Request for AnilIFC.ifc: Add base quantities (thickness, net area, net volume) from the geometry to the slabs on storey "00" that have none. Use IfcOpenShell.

First a look at what the model holds.

```python
import ifcopenshell
import ifcopenshell.util.element
import ifcopenshell.util.unit

model = ifcopenshell.open("AnilIFC.ifc")
print(model.schema)
for unit_type in ("LENGTHUNIT", "AREAUNIT", "VOLUMEUNIT"):
    print(unit_type, ifcopenshell.util.unit.calculate_unit_scale(model, unit_type))
storey = next(s for s in model.by_type("IfcBuildingStorey") if s.Name == "00")
slabs = [e for e in ifcopenshell.util.element.get_decomposition(storey) if e.is_a("IfcSlab")]
for e in sorted(slabs, key=lambda e: e.id()):
    print(e.id(), e.is_a(), e.Name, list(ifcopenshell.util.element.get_psets(e, qtos_only=True)), sep=" | ")
```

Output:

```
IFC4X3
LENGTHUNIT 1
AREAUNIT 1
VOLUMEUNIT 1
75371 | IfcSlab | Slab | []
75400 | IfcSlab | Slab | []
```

```python
import ifcopenshell
import ifcopenshell.api.pset
import ifcopenshell.geom
import ifcopenshell.util.element
import ifcopenshell.util.shape
import ifcopenshell.util.unit

model = ifcopenshell.open("AnilIFC.ifc")
unit_scale = ifcopenshell.util.unit.calculate_unit_scale(model)
area_scale = ifcopenshell.util.unit.calculate_unit_scale(model, "AREAUNIT")
volume_scale = ifcopenshell.util.unit.calculate_unit_scale(model, "VOLUMEUNIT")
settings = ifcopenshell.geom.settings()

storey = next(s for s in model.by_type("IfcBuildingStorey") if s.Name == "00")
slabs = [e for e in ifcopenshell.util.element.get_decomposition(storey) if e.is_a("IfcSlab")]

for e in sorted(slabs, key=lambda e: e.id()):
    if ifcopenshell.util.element.get_psets(e, qtos_only=True, should_inherit=False):
        continue
    # Geometry comes back in metres, in the element's own axes.
    shape = ifcopenshell.geom.create_shape(settings, e)
    values = {
        "Width": ifcopenshell.util.shape.get_z(shape.geometry) / unit_scale,
        "NetArea": ifcopenshell.util.shape.get_footprint_area(shape.geometry) / area_scale,
        "NetVolume": ifcopenshell.util.shape.get_volume(shape.geometry) / volume_scale,
    }
    qto = ifcopenshell.api.pset.add_qto(model, product=e, name="Qto_SlabBaseQuantities")
    ifcopenshell.api.pset.edit_qto(model, qto=qto, properties=values)
    print(e.id(), {k: round(v, 3) for k, v in values.items()})

model.write("AnilIFC_v2.ifc")
```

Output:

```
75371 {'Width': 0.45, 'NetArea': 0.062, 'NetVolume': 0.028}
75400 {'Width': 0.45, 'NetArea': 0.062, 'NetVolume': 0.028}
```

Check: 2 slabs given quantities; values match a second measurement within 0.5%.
